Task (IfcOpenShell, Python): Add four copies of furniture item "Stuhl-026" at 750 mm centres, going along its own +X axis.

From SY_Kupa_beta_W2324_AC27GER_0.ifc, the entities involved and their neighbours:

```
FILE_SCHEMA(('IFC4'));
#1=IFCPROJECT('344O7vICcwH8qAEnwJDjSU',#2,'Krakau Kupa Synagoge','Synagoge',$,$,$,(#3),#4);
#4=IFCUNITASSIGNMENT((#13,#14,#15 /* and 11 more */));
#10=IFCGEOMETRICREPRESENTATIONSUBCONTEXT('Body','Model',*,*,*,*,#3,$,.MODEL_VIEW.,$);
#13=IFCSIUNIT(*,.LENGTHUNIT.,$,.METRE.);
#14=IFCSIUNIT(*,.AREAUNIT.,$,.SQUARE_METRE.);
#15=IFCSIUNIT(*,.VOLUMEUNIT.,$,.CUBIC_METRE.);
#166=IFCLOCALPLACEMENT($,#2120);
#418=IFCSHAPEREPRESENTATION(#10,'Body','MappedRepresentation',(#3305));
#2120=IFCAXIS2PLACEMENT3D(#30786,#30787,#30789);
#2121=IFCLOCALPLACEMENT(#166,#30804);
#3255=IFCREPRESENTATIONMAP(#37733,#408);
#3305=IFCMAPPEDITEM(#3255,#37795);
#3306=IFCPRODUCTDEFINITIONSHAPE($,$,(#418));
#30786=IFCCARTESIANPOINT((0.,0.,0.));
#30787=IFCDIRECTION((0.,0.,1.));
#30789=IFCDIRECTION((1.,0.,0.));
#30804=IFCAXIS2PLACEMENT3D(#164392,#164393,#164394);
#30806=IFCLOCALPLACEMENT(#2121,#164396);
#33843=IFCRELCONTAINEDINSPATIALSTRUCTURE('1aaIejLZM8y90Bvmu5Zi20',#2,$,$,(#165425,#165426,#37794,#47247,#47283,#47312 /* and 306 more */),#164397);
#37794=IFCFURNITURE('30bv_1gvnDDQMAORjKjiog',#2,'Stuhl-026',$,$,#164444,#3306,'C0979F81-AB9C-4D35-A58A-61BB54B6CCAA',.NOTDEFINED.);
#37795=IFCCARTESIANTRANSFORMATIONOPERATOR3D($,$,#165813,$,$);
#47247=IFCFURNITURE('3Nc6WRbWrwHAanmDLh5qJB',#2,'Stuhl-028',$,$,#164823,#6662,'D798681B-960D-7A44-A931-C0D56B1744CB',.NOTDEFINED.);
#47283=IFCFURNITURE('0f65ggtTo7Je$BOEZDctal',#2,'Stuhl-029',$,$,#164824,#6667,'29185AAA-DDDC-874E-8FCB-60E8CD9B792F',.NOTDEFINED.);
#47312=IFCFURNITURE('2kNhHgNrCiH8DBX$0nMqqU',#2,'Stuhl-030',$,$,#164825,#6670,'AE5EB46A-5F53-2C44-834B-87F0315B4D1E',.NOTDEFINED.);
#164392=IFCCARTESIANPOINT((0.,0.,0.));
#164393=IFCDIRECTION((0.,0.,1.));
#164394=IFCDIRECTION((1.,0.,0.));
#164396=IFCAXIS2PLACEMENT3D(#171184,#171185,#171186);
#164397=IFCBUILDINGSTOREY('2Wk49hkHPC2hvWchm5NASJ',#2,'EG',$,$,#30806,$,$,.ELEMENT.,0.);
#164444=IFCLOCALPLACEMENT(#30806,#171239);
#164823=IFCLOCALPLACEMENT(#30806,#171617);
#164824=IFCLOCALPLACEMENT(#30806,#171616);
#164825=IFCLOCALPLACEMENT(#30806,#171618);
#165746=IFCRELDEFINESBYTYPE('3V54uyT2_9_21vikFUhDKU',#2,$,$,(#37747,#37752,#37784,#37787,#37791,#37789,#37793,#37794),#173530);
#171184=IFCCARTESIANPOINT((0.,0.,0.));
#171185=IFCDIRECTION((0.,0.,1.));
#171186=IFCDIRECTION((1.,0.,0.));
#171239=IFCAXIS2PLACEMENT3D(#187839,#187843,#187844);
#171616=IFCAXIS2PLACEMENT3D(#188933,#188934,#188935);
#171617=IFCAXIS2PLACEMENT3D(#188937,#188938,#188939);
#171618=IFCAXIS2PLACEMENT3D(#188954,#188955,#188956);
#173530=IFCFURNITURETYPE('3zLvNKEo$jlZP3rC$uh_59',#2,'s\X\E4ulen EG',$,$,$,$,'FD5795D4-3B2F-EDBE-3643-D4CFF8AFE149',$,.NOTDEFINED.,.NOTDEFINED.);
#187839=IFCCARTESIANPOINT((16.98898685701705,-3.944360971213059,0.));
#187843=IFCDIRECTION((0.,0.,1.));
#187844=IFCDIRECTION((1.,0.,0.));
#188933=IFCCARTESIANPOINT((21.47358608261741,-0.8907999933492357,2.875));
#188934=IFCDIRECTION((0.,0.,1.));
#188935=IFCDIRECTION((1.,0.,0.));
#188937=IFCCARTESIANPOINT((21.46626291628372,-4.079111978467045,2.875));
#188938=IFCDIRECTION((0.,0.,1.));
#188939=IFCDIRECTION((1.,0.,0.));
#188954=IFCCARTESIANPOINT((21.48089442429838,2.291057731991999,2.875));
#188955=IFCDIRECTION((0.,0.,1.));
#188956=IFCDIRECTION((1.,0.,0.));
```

```python
import ifcopenshell
import ifcopenshell.api.geometry
import ifcopenshell.api.root
import ifcopenshell.util.element
import ifcopenshell.util.placement
import ifcopenshell.util.unit

model = ifcopenshell.open("SY_Kupa_beta_W2324_AC27GER_0.ifc")
unit_scale = ifcopenshell.util.unit.calculate_unit_scale(model)


def reuse_history(source, copy):
    """copy_class also copies each property set's owner history, people and application; keep the originals."""
    for rel in copy.IsDefinedBy:
        if rel.is_a("IfcRelDefinesByProperties") and (history := rel.RelatingPropertyDefinition.OwnerHistory):
            rel.RelatingPropertyDefinition.OwnerHistory = source.OwnerHistory
            ifcopenshell.util.element.remove_deep2(model, history)


source = model.by_id(37794)
base = ifcopenshell.util.placement.get_local_placement(source.ObjectPlacement)
step = base[:3, 0] * 0.75 / unit_scale

for i in range(1, 5):
    copy = ifcopenshell.api.root.copy_class(model, product=source)
    copy.Representation = ifcopenshell.util.element.copy_deep(
        model, source.Representation, exclude=["IfcGeometricRepresentationContext", "IfcRepresentationMap"]
    )
    copy.Tag = None
    reuse_history(source, copy)
    matrix = base.copy()
    matrix[:3, 3] += i * step
    print("added at", matrix[:3, 3].round(3) + 0.0)
    ifcopenshell.api.geometry.edit_object_placement(model, product=copy, matrix=matrix, is_si=False)

model.write("SY_Kupa_beta_W2324_AC27GER_0_edited.ifc")
```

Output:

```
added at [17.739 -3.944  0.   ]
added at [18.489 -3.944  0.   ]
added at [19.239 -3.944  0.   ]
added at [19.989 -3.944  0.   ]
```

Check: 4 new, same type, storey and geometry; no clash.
